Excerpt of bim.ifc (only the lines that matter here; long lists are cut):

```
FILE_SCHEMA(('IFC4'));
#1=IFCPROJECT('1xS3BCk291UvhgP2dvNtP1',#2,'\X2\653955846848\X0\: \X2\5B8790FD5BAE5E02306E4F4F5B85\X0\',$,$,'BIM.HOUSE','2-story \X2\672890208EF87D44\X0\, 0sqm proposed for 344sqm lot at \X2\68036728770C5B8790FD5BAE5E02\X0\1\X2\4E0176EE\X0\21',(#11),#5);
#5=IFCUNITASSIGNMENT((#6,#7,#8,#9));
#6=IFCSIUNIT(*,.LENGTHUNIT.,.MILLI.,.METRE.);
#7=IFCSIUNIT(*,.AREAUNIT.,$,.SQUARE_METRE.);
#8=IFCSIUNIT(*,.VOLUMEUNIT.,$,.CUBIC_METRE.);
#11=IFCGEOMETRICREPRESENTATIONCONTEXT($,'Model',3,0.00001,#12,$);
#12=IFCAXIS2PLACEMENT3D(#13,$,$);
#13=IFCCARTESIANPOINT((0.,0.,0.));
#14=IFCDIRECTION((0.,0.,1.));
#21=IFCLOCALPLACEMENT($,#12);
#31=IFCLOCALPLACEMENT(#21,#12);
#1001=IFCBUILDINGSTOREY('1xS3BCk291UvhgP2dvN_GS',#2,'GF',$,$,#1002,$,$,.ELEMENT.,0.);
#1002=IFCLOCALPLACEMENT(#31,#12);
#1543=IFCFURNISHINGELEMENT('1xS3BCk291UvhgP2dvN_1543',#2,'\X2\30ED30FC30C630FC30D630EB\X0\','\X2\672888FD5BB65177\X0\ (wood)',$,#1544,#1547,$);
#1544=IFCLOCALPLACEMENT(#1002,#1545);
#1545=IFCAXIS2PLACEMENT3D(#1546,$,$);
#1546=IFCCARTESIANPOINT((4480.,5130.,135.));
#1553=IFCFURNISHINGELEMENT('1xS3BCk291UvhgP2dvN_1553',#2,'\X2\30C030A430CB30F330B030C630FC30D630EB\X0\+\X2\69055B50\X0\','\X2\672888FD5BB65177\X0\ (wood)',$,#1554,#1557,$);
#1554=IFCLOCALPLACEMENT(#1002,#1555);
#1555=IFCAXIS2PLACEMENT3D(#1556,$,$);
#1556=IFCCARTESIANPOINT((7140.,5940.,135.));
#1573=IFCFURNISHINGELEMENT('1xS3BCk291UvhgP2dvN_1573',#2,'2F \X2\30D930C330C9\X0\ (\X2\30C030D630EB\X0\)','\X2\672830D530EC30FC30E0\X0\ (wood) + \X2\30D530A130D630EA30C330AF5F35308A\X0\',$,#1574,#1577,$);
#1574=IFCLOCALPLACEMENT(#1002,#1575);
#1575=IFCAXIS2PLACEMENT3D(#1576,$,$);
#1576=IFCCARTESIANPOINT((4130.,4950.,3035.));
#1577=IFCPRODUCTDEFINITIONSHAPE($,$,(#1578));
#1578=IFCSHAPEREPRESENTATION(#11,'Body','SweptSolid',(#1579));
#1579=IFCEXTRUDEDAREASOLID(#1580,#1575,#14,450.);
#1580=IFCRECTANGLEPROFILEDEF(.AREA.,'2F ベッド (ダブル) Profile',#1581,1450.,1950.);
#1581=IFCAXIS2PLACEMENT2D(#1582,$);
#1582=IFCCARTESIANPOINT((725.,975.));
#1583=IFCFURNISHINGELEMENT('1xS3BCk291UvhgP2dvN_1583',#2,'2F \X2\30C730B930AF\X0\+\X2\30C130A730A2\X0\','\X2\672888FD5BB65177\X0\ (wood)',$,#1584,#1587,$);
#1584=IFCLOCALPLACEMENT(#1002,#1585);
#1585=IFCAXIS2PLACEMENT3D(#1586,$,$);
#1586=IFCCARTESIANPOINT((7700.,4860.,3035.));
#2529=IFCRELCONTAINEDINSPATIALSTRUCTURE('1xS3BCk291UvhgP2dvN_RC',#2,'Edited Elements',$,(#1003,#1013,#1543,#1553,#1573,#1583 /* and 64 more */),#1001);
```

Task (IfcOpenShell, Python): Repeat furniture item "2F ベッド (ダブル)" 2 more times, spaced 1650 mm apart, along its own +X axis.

```python
import ifcopenshell
import ifcopenshell.api.geometry
import ifcopenshell.api.root
import ifcopenshell.util.element
import ifcopenshell.util.placement
import ifcopenshell.util.unit

model = ifcopenshell.open("bim.ifc")
unit_scale = ifcopenshell.util.unit.calculate_unit_scale(model)


def reuse_history(source, copy):
    """copy_class also copies each property set's owner history, people and application; keep the originals."""
    for rel in copy.IsDefinedBy:
        if rel.is_a("IfcRelDefinesByProperties") and (history := rel.RelatingPropertyDefinition.OwnerHistory):
            rel.RelatingPropertyDefinition.OwnerHistory = source.OwnerHistory
            ifcopenshell.util.element.remove_deep2(model, history)


source = model.by_guid("1xS3BCk291UvhgP2dvN_1573")
base = ifcopenshell.util.placement.get_local_placement(source.ObjectPlacement)
step = base[:3, 0] * 1.65 / unit_scale

for i in range(1, 3):
    copy = ifcopenshell.api.root.copy_class(model, product=source)
    copy.Representation = ifcopenshell.util.element.copy_deep(
        model, source.Representation, exclude=["IfcGeometricRepresentationContext", "IfcRepresentationMap"]
    )
    reuse_history(source, copy)
    matrix = base.copy()
    matrix[:3, 3] += i * step
    print("added at", matrix[:3, 3].round(3) + 0.0)
    ifcopenshell.api.geometry.edit_object_placement(model, product=copy, matrix=matrix, is_si=False)

model.write("bim_rev.ifc")
```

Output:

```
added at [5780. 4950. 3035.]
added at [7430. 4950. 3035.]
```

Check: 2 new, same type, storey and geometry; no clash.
